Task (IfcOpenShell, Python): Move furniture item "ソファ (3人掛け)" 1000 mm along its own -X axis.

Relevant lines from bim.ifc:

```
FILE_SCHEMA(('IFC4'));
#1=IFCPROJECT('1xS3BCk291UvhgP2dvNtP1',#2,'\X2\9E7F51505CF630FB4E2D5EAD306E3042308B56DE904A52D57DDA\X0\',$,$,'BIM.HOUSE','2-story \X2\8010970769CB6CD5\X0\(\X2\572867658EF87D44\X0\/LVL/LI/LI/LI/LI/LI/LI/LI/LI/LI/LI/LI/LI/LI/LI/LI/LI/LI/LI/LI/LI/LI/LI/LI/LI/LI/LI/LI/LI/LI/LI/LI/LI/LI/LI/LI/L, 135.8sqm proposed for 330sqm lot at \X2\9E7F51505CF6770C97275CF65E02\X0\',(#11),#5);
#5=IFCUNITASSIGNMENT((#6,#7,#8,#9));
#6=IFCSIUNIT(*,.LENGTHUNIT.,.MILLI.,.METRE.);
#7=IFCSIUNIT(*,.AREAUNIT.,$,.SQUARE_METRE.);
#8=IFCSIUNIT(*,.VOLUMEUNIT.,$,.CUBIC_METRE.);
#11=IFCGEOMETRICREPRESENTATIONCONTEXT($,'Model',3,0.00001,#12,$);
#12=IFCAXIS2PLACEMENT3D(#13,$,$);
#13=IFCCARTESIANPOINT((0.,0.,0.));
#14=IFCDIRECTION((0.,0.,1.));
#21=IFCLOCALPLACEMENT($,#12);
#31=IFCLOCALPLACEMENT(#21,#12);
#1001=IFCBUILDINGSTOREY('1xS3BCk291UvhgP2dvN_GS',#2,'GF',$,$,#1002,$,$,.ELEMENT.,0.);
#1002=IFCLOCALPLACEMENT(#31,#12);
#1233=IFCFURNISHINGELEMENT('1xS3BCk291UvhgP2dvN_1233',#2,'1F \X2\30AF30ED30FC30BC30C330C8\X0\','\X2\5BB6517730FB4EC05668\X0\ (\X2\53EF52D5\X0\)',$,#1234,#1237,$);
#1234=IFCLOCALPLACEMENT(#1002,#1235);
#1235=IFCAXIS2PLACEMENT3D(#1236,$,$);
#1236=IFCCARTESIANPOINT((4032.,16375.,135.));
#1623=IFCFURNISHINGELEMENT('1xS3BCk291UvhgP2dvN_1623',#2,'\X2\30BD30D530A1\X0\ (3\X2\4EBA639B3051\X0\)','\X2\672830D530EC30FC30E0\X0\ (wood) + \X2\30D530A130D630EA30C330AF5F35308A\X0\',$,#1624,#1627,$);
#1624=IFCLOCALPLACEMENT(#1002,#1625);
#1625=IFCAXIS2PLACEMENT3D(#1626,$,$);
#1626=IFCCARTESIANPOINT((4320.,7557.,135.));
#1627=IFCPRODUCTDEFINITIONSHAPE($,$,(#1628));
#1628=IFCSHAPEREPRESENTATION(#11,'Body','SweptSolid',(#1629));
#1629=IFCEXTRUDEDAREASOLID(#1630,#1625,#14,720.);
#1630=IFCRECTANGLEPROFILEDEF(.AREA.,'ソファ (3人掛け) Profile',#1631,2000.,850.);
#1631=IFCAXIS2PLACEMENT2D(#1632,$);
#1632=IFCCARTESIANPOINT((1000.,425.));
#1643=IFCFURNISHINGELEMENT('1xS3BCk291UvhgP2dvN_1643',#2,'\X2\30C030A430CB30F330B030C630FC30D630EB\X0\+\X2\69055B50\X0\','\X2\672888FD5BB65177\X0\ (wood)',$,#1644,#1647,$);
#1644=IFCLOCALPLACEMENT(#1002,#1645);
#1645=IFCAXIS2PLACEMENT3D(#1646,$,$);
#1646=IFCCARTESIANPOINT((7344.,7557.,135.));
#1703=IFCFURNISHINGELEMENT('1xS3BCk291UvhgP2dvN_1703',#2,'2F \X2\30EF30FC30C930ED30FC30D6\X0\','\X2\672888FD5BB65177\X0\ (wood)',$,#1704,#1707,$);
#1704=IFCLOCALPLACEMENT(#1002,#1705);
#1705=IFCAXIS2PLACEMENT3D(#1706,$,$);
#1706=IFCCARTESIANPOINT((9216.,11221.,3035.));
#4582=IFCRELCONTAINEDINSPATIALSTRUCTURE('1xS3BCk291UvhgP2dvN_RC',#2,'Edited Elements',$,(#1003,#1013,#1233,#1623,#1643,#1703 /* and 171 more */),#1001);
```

```python
import ifcopenshell
import ifcopenshell.api.geometry
import ifcopenshell.util.placement
import ifcopenshell.util.unit

model = ifcopenshell.open("bim.ifc")
unit_scale = ifcopenshell.util.unit.calculate_unit_scale(model)

item = model.by_guid("1xS3BCk291UvhgP2dvN_1623")
matrix = ifcopenshell.util.placement.get_local_placement(item.ObjectPlacement)
matrix[:3, 3] -= matrix[:3, 0] * 1 / unit_scale
ifcopenshell.api.geometry.edit_object_placement(model, product=item, matrix=matrix, is_si=False)

print(ifcopenshell.util.placement.get_local_placement(item.ObjectPlacement).round(3) + 0.0)

model.write("bim_edited.ifc")
```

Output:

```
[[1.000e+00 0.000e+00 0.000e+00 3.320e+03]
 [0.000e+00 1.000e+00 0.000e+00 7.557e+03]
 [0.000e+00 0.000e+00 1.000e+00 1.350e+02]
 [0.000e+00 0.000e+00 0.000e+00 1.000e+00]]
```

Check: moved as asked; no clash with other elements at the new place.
